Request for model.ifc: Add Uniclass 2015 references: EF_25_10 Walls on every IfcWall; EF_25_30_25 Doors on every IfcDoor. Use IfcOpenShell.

First a look at what the model holds.

```python
import ifcopenshell

model = ifcopenshell.open("model.ifc")
print(model.schema)
print("classifications:", [c.Name for c in model.by_type("IfcClassification")])
for ifc_class in ("IfcDoor", "IfcRoof", "IfcStair", "IfcWall", "IfcWindow"):
    print(ifc_class, len(model.by_type(ifc_class)))
```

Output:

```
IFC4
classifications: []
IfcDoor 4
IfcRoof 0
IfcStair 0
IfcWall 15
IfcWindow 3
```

```python
import ifcopenshell
import ifcopenshell.api.classification

model = ifcopenshell.open("model.ifc")

system = ifcopenshell.api.classification.add_classification(model, classification="Uniclass 2015")

codes = {
    "IfcWall": ("EF_25_10", "Walls"),
    "IfcDoor": ("EF_25_30_25", "Doors"),
}
for ifc_class, (code, name) in codes.items():
    products = model.by_type(ifc_class)
    ifcopenshell.api.classification.add_reference(
        model, products=products, classification=system, identification=code, name=name
    )
    print(code, len(products))

model.write("model_edited.ifc")
```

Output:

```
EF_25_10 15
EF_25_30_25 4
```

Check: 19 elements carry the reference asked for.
